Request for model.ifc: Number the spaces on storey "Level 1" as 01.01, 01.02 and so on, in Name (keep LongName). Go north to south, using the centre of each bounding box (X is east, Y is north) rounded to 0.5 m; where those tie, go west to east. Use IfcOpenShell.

First a look at what the model holds.

```python
import ifcopenshell
import ifcopenshell.util.element
import ifcopenshell.util.placement

model = ifcopenshell.open("model.ifc")
print(model.schema)
storey = next(s for s in model.by_type("IfcBuildingStorey") if s.Name == "Level 1")
spaces = [e for e in ifcopenshell.util.element.get_decomposition(storey) if e.is_a("IfcSpace")]
for e in sorted(spaces, key=lambda e: e.id()):
    origin = ifcopenshell.util.placement.get_local_placement(e.ObjectPlacement)[:3, 3]
    print(e.id(), e.Name, e.LongName, origin.round(2) + 0.0, sep=" | ")
```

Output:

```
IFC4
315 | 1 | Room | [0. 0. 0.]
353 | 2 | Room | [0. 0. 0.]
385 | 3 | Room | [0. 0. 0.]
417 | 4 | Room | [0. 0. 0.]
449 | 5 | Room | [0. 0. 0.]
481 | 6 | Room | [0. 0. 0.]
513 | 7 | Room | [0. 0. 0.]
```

```python
import ifcopenshell
import ifcopenshell.geom
import ifcopenshell.util.element
import ifcopenshell.util.shape

model = ifcopenshell.open("model.ifc")
settings = ifcopenshell.geom.settings()
settings.set("use-world-coords", True)


def centre(element):
    shape = ifcopenshell.geom.create_shape(settings, element)
    return ifcopenshell.util.shape.get_bbox_centroid(shape.geometry)


storey = next(s for s in model.by_type("IfcBuildingStorey") if s.Name == "Level 1")
spaces = [e for e in ifcopenshell.util.element.get_decomposition(storey) if e.is_a("IfcSpace")]

# Insertion points can sit at a corner or the storey origin, so sort by the geometry (in metres).
centres = {e: centre(e) for e in spaces}
spaces.sort(key=lambda e: (-round(centres[e][1] / 0.5), centres[e][0]))

for i, e in enumerate(spaces, start=1):
    number = f"01.{i:02d}"
    e.Name = number
    print(e.id(), number)

model.write("model_updated.ifc")
```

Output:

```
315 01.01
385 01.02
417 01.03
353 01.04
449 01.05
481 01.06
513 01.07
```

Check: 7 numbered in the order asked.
